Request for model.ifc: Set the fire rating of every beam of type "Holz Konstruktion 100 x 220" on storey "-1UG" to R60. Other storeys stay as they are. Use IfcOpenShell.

First a look at what the model holds.

```python
import ifcopenshell
import ifcopenshell.util.element

model = ifcopenshell.open("model.ifc")
print(model.schema)
storey = next(s for s in model.by_type("IfcBuildingStorey") if s.Name == "-1UG")
beams = [e for e in ifcopenshell.util.element.get_decomposition(storey) if e.is_a("IfcBeam")]
seen = {}
for e in beams:
    element_type = ifcopenshell.util.element.get_type(e)
    key = (element_type.Name if element_type != e and element_type else None, ifcopenshell.util.element.get_pset(e, "Pset_BeamCommon", "FireRating"))
    seen[key] = seen.get(key, 0) + 1
for (name, value), count in sorted(seen.items(), key=str):
    print(count, "x", name, "|", value)
```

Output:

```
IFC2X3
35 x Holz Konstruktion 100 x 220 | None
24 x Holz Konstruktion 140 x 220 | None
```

```python
import ifcopenshell
import ifcopenshell.api.pset
import ifcopenshell.util.element

model = ifcopenshell.open("model.ifc")

storey = next(s for s in model.by_type("IfcBuildingStorey") if s.Name == "-1UG")
beams = [e for e in ifcopenshell.util.element.get_decomposition(storey) if e.is_a("IfcBeam")]

count = 0
for e in beams:
    element_type = ifcopenshell.util.element.get_type(e)
    if element_type in (None, e) or element_type.Name != "Holz Konstruktion 100 x 220":
        continue
    found = ifcopenshell.util.element.get_pset(e, "Pset_BeamCommon", should_inherit=False)
    if found:
        pset = model.by_id(found["id"])
        if len(ifcopenshell.util.element.get_elements_by_pset(pset)) > 1:
            pset = ifcopenshell.api.pset.unshare_pset(model, products=[e], pset=pset)[0]
    else:
        pset = ifcopenshell.api.pset.add_pset(model, product=e, name="Pset_BeamCommon")
    ifcopenshell.api.pset.edit_pset(model, pset=pset, properties={"FireRating": "R60"})
    count += 1

print(count, "beams updated")

model.write("model_edited.ifc")
```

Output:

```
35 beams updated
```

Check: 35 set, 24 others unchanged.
